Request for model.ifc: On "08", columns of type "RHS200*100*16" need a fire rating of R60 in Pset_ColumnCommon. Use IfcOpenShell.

First a look at what the model holds.

```python
import ifcopenshell
import ifcopenshell.util.element

model = ifcopenshell.open("model.ifc")
print(model.schema)
storey = next(s for s in model.by_type("IfcBuildingStorey") if s.Name == "08")
columns = [e for e in ifcopenshell.util.element.get_decomposition(storey) if e.is_a("IfcColumn")]
seen = {}
for e in columns:
    element_type = ifcopenshell.util.element.get_type(e)
    key = (element_type.Name if element_type != e and element_type else None, ifcopenshell.util.element.get_pset(e, "Pset_ColumnCommon", "FireRating"))
    seen[key] = seen.get(key, 0) + 1
for (name, value), count in sorted(seen.items(), key=str):
    print(count, "x", name, "|", value)
```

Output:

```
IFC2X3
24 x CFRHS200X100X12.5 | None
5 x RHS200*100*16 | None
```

```python
import ifcopenshell
import ifcopenshell.api.pset
import ifcopenshell.util.element

model = ifcopenshell.open("model.ifc")

storey = next(s for s in model.by_type("IfcBuildingStorey") if s.Name == "08")
columns = [e for e in ifcopenshell.util.element.get_decomposition(storey) if e.is_a("IfcColumn")]

count = 0
for e in columns:
    element_type = ifcopenshell.util.element.get_type(e)
    if element_type in (None, e) or element_type.Name != "RHS200*100*16":
        continue
    found = ifcopenshell.util.element.get_pset(e, "Pset_ColumnCommon", should_inherit=False)
    if found:
        pset = model.by_id(found["id"])
        if len(ifcopenshell.util.element.get_elements_by_pset(pset)) > 1:
            pset = ifcopenshell.api.pset.unshare_pset(model, products=[e], pset=pset)[0]
    else:
        pset = ifcopenshell.api.pset.add_pset(model, product=e, name="Pset_ColumnCommon")
    ifcopenshell.api.pset.edit_pset(model, pset=pset, properties={"FireRating": "R60"})
    count += 1

print(count, "columns updated")

model.write("model_rev.ifc")
```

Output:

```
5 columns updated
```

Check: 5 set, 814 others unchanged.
